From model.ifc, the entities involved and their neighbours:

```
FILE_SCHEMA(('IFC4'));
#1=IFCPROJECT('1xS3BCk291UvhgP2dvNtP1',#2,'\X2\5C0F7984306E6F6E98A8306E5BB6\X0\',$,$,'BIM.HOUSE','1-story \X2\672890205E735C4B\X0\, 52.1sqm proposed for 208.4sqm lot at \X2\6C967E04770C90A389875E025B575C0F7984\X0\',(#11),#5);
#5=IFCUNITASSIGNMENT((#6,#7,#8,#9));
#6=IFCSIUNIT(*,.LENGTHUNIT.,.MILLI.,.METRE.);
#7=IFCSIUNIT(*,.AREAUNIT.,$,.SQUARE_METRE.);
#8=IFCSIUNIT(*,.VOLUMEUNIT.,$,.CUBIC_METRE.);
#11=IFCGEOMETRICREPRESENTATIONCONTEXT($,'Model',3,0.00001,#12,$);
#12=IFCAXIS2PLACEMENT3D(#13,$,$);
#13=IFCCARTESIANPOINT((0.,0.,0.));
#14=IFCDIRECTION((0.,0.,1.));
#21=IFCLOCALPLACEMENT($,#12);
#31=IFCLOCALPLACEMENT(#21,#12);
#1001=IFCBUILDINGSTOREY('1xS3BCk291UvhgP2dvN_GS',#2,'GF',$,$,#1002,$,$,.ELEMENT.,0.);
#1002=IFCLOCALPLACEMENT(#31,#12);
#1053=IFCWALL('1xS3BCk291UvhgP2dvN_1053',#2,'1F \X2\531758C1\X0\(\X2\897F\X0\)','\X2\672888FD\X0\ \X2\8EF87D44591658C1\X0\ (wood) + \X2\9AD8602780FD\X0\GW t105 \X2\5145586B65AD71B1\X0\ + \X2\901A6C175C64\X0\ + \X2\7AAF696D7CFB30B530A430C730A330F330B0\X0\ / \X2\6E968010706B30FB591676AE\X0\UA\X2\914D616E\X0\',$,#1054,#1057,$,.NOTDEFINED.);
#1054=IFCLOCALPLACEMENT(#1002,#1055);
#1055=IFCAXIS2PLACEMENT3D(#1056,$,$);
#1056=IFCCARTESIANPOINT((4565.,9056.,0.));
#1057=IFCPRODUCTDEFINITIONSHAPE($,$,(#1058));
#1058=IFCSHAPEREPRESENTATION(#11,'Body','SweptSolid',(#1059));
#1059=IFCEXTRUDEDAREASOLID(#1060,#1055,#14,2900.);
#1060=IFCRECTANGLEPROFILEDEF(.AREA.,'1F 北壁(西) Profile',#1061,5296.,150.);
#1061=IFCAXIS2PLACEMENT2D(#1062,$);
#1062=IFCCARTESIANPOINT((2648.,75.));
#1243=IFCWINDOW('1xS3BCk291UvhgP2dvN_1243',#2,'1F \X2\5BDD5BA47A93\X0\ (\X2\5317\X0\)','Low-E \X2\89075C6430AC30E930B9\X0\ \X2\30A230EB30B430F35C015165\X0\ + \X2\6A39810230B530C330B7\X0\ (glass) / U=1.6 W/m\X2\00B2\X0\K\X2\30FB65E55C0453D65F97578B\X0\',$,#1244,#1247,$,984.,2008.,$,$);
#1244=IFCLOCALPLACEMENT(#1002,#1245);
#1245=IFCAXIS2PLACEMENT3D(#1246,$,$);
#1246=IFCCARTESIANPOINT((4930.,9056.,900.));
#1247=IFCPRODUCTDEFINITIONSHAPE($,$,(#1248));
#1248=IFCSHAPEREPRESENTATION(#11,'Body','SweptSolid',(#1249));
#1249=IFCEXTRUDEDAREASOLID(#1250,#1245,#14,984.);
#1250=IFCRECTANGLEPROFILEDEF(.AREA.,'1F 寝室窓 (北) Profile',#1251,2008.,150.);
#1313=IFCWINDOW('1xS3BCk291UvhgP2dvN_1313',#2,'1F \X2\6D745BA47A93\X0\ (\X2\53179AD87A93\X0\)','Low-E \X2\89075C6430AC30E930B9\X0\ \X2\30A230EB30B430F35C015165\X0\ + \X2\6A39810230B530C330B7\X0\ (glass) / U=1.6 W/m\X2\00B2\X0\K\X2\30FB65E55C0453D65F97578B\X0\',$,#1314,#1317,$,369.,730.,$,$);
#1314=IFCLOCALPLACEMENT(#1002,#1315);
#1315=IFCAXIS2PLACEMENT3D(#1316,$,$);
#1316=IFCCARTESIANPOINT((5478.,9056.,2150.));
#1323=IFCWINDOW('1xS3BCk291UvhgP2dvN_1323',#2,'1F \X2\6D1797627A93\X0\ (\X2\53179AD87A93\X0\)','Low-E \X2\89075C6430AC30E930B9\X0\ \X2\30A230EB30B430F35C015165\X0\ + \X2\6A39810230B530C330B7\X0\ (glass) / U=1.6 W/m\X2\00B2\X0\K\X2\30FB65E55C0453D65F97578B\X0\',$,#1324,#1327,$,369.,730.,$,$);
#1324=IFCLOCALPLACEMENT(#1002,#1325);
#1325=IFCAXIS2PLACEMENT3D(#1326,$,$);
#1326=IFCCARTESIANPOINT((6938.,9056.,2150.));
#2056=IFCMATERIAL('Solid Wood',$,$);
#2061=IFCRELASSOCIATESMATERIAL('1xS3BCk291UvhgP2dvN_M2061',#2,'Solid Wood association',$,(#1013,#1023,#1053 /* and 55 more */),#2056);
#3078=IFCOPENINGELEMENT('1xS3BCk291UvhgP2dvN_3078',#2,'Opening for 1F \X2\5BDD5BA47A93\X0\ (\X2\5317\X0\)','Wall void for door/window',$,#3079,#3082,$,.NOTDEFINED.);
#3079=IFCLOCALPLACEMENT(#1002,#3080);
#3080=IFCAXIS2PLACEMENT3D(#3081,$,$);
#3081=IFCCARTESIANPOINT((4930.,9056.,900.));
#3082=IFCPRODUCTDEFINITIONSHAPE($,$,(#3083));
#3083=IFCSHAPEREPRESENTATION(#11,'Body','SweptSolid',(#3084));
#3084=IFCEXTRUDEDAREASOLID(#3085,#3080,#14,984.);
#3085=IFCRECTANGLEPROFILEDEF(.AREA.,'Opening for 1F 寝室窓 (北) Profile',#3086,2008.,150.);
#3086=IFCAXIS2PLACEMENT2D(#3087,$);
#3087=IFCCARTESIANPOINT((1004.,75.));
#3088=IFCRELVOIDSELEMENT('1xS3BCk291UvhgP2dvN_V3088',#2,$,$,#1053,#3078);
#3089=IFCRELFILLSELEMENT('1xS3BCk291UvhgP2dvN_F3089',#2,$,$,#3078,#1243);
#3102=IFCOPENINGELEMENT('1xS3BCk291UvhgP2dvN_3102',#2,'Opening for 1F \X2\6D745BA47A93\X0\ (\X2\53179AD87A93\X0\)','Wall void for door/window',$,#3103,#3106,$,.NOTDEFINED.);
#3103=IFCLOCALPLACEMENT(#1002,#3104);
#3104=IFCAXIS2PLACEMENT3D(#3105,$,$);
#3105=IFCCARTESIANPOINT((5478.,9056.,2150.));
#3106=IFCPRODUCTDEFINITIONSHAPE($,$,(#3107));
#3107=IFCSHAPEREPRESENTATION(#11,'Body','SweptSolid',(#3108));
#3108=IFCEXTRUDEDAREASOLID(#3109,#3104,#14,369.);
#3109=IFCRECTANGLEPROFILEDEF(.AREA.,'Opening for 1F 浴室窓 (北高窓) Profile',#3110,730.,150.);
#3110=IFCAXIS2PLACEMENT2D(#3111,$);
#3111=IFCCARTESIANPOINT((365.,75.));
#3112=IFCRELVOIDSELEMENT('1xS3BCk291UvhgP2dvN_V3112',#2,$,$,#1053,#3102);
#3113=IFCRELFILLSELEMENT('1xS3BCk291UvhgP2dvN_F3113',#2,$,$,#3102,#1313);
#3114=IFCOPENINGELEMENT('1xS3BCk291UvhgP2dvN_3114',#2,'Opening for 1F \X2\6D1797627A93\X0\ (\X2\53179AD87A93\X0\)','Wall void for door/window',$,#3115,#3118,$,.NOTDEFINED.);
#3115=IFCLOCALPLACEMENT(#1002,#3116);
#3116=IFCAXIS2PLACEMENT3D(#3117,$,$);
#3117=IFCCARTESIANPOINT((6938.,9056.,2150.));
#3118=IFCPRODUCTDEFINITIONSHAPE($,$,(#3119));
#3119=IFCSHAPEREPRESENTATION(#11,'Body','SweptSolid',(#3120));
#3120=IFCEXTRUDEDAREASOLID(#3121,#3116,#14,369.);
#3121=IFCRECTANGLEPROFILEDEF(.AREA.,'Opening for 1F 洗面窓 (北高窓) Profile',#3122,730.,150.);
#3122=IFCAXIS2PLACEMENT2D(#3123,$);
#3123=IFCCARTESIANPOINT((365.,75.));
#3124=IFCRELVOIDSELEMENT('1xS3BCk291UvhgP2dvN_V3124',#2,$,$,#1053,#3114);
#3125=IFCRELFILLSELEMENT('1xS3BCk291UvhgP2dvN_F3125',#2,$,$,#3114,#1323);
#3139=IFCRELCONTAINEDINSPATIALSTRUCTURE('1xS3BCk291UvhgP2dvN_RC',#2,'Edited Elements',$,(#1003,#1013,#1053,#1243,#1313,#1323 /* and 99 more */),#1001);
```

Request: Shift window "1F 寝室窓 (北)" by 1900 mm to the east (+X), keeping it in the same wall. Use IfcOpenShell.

```python
import ifcopenshell
import ifcopenshell.api.geometry
import ifcopenshell.util.placement

model = ifcopenshell.open("model.ifc")

window = model.by_guid("1xS3BCk291UvhgP2dvN_1243")
opening = window.FillsVoids[0].RelatingOpeningElement
wall = opening.VoidsElements[0].RelatingBuildingElement

wall_matrix = ifcopenshell.util.placement.get_local_placement(wall.ObjectPlacement)
shift = wall_matrix[:3, 0] * 1900.0
before = ifcopenshell.util.placement.get_local_placement(window.ObjectPlacement)[:3, 3].copy()

# The window is not placed relative to its opening, so move both.
for product in (opening, window):
    matrix = ifcopenshell.util.placement.get_local_placement(product.ObjectPlacement)
    matrix[:3, 3] += shift
    ifcopenshell.api.geometry.edit_object_placement(model, product=product, matrix=matrix, is_si=False)

after = ifcopenshell.util.placement.get_local_placement(window.ObjectPlacement)[:3, 3]
print("window moved by", (after - before).round(3) + 0.0)

model.write("model_rev.ifc")
```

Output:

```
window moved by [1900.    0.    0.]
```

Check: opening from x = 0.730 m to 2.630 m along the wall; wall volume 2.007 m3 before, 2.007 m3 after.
